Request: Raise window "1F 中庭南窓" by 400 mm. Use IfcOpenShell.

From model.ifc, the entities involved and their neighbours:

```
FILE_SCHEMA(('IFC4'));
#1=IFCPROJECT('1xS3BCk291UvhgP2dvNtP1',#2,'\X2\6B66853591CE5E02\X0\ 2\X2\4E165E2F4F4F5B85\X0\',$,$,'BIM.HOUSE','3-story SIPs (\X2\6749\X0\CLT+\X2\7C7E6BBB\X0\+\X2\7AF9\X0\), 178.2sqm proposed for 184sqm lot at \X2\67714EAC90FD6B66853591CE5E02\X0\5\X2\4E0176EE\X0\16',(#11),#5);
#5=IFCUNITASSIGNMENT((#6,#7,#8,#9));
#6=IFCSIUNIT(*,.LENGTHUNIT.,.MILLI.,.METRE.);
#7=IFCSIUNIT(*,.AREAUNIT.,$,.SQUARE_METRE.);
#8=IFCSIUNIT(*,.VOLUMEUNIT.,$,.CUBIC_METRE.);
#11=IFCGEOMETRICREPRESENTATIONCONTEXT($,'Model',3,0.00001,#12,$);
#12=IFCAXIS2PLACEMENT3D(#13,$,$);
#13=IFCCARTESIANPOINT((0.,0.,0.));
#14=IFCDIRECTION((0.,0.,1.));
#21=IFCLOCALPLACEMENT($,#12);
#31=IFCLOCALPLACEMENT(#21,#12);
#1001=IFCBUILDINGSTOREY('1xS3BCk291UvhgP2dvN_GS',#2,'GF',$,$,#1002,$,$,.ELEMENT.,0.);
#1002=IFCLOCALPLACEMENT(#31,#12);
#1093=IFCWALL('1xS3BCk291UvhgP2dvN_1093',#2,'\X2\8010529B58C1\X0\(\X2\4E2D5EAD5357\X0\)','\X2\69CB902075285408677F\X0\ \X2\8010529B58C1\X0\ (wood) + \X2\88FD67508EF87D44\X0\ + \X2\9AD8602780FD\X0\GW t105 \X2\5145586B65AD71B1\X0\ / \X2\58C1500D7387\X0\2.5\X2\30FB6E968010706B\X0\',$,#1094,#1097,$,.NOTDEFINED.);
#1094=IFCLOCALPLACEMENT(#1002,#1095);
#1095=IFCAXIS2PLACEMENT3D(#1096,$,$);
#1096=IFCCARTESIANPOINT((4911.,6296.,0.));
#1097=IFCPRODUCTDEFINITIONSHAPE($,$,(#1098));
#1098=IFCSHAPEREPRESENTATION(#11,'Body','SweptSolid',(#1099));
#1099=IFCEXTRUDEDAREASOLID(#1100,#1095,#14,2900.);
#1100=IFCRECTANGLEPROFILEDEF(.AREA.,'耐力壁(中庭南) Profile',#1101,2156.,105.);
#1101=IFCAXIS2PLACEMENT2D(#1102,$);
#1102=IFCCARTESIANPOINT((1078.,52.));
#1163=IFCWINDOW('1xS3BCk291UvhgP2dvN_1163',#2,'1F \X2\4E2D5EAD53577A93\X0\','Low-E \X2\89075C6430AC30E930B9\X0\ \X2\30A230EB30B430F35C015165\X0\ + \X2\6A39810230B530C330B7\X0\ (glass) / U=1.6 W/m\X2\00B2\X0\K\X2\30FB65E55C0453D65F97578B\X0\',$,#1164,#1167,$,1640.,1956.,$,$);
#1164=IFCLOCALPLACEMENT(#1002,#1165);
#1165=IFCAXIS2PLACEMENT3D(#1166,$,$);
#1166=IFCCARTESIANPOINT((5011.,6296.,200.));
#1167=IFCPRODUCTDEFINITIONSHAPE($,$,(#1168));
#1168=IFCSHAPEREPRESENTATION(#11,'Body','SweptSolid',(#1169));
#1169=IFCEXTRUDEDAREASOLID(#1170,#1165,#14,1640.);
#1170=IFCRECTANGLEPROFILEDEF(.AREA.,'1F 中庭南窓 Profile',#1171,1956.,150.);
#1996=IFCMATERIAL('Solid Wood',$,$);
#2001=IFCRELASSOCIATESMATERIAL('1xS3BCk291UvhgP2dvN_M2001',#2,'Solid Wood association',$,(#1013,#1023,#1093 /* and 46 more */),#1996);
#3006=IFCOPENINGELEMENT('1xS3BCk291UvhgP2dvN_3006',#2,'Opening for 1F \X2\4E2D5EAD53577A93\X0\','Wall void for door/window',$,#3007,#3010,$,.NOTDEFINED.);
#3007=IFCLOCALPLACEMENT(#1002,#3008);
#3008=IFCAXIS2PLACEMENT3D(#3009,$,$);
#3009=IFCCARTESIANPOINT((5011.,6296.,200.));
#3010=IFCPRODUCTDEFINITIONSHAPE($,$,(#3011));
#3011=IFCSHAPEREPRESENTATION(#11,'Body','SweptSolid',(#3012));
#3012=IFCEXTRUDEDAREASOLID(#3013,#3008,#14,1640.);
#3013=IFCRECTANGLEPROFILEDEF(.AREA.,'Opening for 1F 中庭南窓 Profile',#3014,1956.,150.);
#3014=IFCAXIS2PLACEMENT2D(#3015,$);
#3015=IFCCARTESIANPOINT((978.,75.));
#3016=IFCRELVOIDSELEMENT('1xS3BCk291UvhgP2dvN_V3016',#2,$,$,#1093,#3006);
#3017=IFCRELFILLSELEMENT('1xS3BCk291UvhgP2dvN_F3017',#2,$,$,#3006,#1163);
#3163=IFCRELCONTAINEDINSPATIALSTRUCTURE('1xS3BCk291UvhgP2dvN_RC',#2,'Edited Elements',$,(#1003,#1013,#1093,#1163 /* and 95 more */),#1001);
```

```python
import numpy as np
import ifcopenshell
import ifcopenshell.api.geometry
import ifcopenshell.util.placement
import ifcopenshell.util.unit

model = ifcopenshell.open("model.ifc")
unit_scale = ifcopenshell.util.unit.calculate_unit_scale(model)

window = model.by_id(1163)
opening = window.FillsVoids[0].RelatingOpeningElement
dz = 0.4 / unit_scale

shift = np.array([0.0, 0.0, dz])
# The window is not placed relative to its opening, so move both.
for product in (opening, window):
    matrix = ifcopenshell.util.placement.get_local_placement(product.ObjectPlacement)
    matrix[:3, 3] += shift
    ifcopenshell.api.geometry.edit_object_placement(model, product=product, matrix=matrix, is_si=False)

print(f"moved by {dz * unit_scale:+.3f} m")

model.write("model_updated.ifc")
```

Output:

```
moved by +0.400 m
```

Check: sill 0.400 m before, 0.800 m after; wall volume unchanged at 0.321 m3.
